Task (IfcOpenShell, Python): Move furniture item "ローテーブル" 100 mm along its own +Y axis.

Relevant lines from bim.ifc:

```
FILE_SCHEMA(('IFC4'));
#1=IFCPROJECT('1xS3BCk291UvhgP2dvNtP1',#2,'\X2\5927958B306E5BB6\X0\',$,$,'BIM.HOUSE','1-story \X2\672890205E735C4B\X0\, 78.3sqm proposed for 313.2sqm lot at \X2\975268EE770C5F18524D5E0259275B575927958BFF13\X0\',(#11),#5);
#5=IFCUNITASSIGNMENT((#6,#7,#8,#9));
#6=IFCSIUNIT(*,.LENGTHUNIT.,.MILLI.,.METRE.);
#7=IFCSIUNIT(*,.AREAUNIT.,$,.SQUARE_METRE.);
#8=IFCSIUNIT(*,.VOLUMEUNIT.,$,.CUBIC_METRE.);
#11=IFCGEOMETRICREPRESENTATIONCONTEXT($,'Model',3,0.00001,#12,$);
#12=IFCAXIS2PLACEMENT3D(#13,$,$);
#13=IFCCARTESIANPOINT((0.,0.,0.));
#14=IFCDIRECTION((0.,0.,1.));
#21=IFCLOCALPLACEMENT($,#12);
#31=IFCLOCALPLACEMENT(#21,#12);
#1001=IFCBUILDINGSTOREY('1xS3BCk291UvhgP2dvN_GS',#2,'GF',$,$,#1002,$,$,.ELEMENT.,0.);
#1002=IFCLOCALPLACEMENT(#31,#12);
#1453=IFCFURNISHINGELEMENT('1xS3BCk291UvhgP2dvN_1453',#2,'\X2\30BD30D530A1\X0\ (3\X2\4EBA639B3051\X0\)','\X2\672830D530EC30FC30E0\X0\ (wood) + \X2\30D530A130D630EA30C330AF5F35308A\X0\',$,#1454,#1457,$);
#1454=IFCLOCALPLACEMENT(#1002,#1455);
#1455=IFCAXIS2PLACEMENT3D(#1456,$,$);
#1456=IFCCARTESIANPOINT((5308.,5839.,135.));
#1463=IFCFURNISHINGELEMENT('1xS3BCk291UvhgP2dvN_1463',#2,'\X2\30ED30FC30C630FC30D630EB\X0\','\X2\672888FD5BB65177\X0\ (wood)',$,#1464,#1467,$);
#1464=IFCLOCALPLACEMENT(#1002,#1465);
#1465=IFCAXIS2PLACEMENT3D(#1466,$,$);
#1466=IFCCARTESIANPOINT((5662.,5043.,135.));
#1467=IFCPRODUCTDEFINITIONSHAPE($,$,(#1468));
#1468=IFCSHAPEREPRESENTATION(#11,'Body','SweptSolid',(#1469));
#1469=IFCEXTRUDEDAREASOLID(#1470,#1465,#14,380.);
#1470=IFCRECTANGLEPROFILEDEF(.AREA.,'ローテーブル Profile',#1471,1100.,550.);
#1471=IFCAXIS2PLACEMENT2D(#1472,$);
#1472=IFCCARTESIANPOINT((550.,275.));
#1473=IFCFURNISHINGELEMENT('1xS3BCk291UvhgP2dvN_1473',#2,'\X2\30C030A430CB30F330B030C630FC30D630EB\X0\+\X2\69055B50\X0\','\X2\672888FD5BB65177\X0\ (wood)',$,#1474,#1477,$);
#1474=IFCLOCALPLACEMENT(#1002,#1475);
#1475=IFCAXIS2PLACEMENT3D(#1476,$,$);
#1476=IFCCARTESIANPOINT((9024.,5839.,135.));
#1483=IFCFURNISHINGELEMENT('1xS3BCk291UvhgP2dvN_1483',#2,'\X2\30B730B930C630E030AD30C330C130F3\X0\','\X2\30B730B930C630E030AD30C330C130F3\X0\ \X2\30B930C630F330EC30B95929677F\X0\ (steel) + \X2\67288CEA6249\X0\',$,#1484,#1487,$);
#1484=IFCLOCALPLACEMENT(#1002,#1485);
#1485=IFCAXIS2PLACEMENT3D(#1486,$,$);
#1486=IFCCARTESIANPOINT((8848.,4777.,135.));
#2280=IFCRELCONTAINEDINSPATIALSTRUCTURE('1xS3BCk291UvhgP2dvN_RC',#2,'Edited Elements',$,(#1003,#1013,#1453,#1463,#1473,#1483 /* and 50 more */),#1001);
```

```python
import ifcopenshell
import ifcopenshell.api.geometry
import ifcopenshell.util.placement
import ifcopenshell.util.unit

model = ifcopenshell.open("bim.ifc")
unit_scale = ifcopenshell.util.unit.calculate_unit_scale(model)

item = model.by_guid("1xS3BCk291UvhgP2dvN_1463")
matrix = ifcopenshell.util.placement.get_local_placement(item.ObjectPlacement)
matrix[:3, 3] += matrix[:3, 1] * 0.1 / unit_scale
ifcopenshell.api.geometry.edit_object_placement(model, product=item, matrix=matrix, is_si=False)

print(ifcopenshell.util.placement.get_local_placement(item.ObjectPlacement).round(3) + 0.0)

model.write("bim_rev.ifc")
```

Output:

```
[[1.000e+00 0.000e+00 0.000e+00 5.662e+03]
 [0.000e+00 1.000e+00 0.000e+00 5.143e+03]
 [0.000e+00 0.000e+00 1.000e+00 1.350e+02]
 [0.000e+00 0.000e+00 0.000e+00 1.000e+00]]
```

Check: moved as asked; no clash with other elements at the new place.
